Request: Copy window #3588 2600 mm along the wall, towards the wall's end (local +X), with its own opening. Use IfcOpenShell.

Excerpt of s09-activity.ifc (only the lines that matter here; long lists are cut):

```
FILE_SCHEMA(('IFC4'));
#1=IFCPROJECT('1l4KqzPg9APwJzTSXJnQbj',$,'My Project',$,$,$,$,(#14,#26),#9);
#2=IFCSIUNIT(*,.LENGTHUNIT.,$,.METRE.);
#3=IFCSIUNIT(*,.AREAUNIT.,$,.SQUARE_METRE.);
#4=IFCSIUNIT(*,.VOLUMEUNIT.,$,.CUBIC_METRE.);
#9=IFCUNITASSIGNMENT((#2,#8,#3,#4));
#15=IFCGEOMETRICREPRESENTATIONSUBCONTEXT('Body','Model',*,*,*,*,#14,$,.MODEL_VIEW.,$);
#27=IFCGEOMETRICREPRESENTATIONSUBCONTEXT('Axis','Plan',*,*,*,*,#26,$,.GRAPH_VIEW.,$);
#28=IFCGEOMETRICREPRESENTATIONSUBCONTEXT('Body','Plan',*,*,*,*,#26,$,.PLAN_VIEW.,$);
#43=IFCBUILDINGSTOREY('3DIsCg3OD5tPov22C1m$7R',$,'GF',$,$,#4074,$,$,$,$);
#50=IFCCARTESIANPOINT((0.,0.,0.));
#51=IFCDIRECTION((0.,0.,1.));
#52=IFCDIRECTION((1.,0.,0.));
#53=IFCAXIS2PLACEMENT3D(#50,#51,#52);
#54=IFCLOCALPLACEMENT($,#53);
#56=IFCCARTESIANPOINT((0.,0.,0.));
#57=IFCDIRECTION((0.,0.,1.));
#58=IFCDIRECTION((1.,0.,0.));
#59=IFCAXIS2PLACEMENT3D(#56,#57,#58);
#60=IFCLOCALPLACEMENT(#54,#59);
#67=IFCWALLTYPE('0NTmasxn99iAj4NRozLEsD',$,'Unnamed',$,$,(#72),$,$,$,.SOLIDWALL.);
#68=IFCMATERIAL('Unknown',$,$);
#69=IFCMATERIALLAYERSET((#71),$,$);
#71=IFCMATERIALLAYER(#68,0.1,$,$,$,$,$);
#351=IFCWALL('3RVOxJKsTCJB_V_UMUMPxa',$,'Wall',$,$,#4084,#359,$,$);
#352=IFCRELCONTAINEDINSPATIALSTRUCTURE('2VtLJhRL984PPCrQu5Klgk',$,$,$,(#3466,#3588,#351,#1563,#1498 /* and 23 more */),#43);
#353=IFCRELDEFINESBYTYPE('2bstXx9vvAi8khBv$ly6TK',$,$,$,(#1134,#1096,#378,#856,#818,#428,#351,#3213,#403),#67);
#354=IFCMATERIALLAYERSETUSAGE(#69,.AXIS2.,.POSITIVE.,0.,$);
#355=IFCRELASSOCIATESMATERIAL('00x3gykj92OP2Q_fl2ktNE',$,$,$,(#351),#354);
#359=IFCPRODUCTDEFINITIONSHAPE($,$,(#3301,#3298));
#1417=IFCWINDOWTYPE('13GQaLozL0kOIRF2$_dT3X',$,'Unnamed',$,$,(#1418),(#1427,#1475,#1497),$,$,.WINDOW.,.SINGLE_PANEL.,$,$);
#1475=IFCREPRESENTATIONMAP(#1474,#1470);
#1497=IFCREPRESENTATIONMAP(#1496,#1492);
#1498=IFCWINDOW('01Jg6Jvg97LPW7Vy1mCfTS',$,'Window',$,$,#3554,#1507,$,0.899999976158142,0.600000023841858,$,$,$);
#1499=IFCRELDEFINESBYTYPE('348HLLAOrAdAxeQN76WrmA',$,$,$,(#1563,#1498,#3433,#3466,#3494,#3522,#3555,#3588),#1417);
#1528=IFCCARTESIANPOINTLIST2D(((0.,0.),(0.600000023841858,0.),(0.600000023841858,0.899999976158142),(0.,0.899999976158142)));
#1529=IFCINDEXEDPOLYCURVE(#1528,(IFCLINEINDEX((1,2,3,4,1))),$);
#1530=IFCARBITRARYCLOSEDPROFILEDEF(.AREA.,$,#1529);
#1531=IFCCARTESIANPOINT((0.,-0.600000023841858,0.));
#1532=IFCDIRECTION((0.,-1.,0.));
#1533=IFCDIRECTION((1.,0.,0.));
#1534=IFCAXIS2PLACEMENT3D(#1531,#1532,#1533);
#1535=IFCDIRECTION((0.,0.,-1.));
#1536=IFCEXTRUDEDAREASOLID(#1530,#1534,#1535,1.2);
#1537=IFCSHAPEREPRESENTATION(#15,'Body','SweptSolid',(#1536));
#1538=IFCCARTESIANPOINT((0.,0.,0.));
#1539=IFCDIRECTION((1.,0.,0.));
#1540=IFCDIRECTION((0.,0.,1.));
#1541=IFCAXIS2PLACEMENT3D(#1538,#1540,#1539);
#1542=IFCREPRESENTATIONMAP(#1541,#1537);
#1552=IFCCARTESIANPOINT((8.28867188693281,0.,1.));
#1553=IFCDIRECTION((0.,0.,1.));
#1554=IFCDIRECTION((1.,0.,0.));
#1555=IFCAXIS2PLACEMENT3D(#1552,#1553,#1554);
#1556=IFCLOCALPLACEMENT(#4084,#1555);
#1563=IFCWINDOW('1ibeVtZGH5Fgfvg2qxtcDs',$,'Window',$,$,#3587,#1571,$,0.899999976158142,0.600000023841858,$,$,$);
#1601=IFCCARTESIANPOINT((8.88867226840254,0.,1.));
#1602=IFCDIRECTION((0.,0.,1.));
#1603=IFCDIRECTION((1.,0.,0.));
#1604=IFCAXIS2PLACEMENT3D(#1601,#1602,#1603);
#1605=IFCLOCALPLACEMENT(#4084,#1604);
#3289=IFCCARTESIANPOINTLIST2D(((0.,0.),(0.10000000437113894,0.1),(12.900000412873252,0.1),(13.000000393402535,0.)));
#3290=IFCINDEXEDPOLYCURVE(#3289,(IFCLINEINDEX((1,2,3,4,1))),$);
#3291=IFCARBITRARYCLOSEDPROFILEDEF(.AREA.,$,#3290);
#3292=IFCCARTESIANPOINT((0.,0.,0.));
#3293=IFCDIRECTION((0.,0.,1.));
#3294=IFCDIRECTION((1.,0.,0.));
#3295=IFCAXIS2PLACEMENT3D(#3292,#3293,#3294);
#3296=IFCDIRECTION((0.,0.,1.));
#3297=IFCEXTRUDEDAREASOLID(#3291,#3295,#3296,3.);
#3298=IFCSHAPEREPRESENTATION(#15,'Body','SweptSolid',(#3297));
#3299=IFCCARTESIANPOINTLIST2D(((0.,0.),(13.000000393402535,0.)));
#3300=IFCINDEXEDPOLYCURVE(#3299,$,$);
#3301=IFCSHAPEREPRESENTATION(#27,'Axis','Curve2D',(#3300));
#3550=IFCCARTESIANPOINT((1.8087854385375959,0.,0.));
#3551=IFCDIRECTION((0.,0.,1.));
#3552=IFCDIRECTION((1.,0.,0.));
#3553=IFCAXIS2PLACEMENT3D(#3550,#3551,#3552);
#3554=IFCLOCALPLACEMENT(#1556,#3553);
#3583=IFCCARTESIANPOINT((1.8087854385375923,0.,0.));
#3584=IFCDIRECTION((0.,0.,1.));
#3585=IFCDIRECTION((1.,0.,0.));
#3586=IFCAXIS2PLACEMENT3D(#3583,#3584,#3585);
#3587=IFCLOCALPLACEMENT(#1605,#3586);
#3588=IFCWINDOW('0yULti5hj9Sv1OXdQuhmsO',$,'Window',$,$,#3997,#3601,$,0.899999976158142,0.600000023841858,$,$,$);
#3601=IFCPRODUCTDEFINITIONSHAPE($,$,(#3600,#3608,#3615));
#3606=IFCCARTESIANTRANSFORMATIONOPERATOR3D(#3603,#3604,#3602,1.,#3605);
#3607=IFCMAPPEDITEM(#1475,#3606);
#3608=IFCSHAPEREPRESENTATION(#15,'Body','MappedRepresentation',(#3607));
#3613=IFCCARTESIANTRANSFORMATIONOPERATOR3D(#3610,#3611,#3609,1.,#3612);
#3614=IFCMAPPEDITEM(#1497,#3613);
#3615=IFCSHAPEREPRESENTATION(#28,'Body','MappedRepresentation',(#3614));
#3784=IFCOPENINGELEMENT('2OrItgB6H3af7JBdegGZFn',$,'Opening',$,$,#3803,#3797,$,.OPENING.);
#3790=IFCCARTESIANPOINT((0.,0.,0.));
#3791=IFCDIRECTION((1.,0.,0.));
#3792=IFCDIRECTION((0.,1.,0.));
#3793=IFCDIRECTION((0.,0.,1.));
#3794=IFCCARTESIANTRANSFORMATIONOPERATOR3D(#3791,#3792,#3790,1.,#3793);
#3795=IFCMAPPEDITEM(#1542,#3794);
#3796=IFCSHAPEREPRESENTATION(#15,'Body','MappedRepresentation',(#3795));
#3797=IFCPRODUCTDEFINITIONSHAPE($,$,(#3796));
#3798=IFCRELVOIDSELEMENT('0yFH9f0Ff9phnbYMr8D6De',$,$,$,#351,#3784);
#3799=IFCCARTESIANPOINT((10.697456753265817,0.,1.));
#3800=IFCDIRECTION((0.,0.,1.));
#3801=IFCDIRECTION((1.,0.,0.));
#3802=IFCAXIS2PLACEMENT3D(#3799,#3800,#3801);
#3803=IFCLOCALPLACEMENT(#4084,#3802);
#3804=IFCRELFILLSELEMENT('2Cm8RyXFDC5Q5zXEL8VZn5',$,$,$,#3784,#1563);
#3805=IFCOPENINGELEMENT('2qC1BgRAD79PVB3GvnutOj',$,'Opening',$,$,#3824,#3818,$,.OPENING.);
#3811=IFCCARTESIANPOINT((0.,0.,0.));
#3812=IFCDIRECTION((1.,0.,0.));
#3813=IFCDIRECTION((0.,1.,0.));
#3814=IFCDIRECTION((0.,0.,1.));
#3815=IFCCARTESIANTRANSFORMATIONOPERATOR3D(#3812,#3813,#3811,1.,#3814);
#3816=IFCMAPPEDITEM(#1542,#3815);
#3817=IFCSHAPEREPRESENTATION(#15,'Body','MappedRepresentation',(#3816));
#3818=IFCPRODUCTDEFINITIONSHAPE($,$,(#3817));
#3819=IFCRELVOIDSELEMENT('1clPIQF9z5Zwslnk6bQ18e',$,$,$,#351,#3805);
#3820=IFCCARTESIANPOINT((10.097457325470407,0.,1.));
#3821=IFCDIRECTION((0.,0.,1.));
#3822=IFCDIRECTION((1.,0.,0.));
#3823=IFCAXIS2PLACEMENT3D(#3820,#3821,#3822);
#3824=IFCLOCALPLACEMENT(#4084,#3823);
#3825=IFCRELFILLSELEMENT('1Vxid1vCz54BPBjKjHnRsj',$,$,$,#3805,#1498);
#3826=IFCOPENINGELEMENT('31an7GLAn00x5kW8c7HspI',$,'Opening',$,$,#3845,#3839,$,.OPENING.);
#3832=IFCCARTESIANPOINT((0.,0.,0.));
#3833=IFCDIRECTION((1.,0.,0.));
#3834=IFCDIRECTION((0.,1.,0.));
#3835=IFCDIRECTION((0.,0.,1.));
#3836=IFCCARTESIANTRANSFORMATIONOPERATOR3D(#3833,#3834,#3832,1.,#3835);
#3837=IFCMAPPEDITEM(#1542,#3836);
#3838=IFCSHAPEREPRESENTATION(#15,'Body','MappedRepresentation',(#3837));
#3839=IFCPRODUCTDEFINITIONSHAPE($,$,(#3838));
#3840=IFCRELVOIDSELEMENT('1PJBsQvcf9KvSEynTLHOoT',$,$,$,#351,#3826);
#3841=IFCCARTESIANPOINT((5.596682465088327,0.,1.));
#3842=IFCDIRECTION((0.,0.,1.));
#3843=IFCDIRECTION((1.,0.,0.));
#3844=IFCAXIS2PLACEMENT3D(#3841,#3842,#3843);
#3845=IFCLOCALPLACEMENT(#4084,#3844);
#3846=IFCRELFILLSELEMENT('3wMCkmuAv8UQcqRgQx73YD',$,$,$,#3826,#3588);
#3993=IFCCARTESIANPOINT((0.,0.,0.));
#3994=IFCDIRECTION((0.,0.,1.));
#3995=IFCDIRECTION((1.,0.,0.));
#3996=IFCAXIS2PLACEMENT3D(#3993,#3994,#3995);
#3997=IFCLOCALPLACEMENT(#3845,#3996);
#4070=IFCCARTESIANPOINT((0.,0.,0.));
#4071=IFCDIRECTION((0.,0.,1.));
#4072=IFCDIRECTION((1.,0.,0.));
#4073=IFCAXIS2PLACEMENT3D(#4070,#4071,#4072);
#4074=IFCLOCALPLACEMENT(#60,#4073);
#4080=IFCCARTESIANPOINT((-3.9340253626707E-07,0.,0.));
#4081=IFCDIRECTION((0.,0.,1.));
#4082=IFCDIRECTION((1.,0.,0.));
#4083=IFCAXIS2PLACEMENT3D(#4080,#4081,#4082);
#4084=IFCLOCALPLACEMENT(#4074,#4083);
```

```python
import ifcopenshell
import ifcopenshell.api.feature
import ifcopenshell.api.geometry
import ifcopenshell.api.root
import ifcopenshell.geom
import ifcopenshell.util.element
import ifcopenshell.util.placement
import ifcopenshell.util.shape
import ifcopenshell.util.unit

model = ifcopenshell.open("s09-activity.ifc")
unit_scale = ifcopenshell.util.unit.calculate_unit_scale(model)
settings = ifcopenshell.geom.settings()


def volume(element):
    """Net volume in cubic metres, openings subtracted."""
    shape = ifcopenshell.geom.create_shape(settings, element)
    return ifcopenshell.util.shape.get_volume(shape.geometry)


window = model.by_id(3588)
opening = window.FillsVoids[0].RelatingOpeningElement
wall = opening.VoidsElements[0].RelatingBuildingElement
before = volume(wall)
shift = ifcopenshell.util.placement.get_local_placement(wall.ObjectPlacement)[:3, 0] * 2.6 / unit_scale

# copy_class copies the void relationship, type, container and properties, but no geometry.
new_opening = ifcopenshell.api.root.copy_class(model, product=opening)
new_opening.Representation = ifcopenshell.util.element.copy_deep(
    model, opening.Representation, exclude=["IfcGeometricRepresentationContext", "IfcRepresentationMap"]
)
new_window = ifcopenshell.api.root.copy_class(model, product=window)
new_window.Representation = ifcopenshell.util.element.copy_deep(
    model, window.Representation, exclude=["IfcGeometricRepresentationContext", "IfcRepresentationMap"]
)
ifcopenshell.api.feature.add_filling(model, opening=new_opening, element=new_window)

for old, new in ((opening, new_opening), (window, new_window)):
    matrix = ifcopenshell.util.placement.get_local_placement(old.ObjectPlacement)
    matrix[:3, 3] += shift
    ifcopenshell.api.geometry.edit_object_placement(model, product=new, matrix=matrix, is_si=False)

after = volume(wall)

print(f"wall volume {before:.3f} -> {after:.3f} m3")

model.write("s09-activity_v2.ifc")
```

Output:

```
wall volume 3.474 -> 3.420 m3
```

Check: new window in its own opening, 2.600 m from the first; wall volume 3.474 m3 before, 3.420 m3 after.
